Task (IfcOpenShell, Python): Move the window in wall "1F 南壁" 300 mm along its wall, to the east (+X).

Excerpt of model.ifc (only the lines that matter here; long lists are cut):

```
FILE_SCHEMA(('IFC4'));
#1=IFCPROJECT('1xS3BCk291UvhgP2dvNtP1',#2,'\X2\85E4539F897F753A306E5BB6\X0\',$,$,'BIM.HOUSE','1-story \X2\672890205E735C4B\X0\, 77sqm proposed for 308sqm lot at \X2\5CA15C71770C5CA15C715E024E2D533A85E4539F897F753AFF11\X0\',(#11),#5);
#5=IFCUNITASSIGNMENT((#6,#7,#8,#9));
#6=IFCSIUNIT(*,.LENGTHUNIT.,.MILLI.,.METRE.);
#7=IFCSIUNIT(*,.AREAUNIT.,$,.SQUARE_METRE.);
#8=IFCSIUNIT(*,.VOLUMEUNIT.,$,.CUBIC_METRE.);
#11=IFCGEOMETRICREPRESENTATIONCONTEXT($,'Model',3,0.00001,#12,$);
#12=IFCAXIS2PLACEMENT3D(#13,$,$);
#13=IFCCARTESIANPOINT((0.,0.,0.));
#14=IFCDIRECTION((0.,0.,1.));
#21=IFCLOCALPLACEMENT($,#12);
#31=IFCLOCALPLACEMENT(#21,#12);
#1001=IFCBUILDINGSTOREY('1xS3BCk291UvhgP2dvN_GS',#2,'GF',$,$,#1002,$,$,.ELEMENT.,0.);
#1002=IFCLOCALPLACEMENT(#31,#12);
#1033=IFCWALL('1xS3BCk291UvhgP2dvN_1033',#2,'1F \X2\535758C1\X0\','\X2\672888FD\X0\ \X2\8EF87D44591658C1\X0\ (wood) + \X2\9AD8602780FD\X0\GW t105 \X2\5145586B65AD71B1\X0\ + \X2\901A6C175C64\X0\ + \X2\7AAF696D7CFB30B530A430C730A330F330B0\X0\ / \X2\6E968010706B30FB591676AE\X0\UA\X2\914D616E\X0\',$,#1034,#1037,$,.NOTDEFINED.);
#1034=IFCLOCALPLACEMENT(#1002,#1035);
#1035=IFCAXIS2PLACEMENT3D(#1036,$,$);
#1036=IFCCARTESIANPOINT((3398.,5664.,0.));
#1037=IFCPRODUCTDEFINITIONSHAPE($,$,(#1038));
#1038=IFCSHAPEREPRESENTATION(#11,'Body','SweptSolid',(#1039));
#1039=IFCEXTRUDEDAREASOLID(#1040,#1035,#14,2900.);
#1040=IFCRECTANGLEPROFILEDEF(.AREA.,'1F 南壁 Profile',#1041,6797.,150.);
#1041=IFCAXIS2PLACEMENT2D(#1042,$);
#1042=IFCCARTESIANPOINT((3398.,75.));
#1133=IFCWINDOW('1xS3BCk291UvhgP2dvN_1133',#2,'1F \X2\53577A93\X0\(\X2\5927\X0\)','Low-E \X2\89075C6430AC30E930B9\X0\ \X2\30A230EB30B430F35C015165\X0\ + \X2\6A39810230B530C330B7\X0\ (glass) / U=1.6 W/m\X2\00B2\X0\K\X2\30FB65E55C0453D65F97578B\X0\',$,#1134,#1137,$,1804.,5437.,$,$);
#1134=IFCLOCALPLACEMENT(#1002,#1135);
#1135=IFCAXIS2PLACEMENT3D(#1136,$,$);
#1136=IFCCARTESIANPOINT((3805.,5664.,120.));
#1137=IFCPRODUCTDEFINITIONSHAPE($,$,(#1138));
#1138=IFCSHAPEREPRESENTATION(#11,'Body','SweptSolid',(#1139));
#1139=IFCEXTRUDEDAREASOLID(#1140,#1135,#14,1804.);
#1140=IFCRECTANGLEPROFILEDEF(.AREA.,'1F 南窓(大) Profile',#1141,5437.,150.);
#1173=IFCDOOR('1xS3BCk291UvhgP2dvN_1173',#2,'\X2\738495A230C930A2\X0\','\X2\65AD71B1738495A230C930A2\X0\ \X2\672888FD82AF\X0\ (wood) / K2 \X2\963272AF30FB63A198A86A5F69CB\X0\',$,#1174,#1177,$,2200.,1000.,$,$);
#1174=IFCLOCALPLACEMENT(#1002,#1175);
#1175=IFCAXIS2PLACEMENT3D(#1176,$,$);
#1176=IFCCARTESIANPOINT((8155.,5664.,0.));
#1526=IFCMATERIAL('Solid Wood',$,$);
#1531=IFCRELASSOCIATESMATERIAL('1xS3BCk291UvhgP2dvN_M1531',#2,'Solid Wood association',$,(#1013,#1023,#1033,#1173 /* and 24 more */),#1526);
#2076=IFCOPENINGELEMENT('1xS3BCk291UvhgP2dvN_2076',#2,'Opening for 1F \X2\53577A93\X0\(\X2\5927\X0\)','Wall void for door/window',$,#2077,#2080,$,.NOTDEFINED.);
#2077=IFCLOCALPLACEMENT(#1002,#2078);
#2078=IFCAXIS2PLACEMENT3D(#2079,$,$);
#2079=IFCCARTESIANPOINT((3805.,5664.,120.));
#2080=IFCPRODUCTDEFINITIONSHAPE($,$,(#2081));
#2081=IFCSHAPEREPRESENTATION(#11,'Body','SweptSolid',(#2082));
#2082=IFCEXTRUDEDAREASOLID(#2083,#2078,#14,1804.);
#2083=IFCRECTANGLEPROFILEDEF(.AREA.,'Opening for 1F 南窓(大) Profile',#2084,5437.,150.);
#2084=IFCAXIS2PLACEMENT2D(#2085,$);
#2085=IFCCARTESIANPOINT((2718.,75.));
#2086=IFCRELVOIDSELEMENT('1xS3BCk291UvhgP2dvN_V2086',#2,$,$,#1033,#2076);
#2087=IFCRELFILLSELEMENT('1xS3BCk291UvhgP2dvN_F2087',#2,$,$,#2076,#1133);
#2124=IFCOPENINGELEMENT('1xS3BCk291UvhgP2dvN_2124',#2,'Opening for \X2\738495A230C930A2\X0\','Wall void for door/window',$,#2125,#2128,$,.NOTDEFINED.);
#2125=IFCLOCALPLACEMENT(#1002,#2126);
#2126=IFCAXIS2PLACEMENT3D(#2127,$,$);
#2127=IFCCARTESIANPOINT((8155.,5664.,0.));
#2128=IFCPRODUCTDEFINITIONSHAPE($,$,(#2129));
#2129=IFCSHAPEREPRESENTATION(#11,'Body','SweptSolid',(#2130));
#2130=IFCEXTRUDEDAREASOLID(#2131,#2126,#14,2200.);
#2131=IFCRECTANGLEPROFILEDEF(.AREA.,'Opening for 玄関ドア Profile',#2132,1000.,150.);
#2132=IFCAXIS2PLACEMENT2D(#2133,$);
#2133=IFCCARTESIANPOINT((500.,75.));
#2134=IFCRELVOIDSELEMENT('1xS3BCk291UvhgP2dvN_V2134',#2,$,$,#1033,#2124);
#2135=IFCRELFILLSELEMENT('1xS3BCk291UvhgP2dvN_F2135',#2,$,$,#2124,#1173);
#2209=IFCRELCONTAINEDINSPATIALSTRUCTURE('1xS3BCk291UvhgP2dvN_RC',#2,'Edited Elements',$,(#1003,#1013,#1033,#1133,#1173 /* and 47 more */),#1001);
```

```python
import ifcopenshell
import ifcopenshell.api.geometry
import ifcopenshell.util.placement
import ifcopenshell.util.unit

model = ifcopenshell.open("model.ifc")
unit_scale = ifcopenshell.util.unit.calculate_unit_scale(model)

window = model.by_guid("1xS3BCk291UvhgP2dvN_1133")
opening = window.FillsVoids[0].RelatingOpeningElement
wall = opening.VoidsElements[0].RelatingBuildingElement

wall_matrix = ifcopenshell.util.placement.get_local_placement(wall.ObjectPlacement)
shift = wall_matrix[:3, 0] * 0.3 / unit_scale
before = ifcopenshell.util.placement.get_local_placement(window.ObjectPlacement)[:3, 3].copy()

# The window is not placed relative to its opening, so move both.
for product in (opening, window):
    matrix = ifcopenshell.util.placement.get_local_placement(product.ObjectPlacement)
    matrix[:3, 3] += shift
    ifcopenshell.api.geometry.edit_object_placement(model, product=product, matrix=matrix, is_si=False)

after = ifcopenshell.util.placement.get_local_placement(window.ObjectPlacement)[:3, 3]
print("window moved by", (after - before).round(3) + 0.0)

model.write("model_edited.ifc")
```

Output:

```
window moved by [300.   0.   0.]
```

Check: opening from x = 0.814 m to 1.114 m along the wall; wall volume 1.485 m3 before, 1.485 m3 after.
